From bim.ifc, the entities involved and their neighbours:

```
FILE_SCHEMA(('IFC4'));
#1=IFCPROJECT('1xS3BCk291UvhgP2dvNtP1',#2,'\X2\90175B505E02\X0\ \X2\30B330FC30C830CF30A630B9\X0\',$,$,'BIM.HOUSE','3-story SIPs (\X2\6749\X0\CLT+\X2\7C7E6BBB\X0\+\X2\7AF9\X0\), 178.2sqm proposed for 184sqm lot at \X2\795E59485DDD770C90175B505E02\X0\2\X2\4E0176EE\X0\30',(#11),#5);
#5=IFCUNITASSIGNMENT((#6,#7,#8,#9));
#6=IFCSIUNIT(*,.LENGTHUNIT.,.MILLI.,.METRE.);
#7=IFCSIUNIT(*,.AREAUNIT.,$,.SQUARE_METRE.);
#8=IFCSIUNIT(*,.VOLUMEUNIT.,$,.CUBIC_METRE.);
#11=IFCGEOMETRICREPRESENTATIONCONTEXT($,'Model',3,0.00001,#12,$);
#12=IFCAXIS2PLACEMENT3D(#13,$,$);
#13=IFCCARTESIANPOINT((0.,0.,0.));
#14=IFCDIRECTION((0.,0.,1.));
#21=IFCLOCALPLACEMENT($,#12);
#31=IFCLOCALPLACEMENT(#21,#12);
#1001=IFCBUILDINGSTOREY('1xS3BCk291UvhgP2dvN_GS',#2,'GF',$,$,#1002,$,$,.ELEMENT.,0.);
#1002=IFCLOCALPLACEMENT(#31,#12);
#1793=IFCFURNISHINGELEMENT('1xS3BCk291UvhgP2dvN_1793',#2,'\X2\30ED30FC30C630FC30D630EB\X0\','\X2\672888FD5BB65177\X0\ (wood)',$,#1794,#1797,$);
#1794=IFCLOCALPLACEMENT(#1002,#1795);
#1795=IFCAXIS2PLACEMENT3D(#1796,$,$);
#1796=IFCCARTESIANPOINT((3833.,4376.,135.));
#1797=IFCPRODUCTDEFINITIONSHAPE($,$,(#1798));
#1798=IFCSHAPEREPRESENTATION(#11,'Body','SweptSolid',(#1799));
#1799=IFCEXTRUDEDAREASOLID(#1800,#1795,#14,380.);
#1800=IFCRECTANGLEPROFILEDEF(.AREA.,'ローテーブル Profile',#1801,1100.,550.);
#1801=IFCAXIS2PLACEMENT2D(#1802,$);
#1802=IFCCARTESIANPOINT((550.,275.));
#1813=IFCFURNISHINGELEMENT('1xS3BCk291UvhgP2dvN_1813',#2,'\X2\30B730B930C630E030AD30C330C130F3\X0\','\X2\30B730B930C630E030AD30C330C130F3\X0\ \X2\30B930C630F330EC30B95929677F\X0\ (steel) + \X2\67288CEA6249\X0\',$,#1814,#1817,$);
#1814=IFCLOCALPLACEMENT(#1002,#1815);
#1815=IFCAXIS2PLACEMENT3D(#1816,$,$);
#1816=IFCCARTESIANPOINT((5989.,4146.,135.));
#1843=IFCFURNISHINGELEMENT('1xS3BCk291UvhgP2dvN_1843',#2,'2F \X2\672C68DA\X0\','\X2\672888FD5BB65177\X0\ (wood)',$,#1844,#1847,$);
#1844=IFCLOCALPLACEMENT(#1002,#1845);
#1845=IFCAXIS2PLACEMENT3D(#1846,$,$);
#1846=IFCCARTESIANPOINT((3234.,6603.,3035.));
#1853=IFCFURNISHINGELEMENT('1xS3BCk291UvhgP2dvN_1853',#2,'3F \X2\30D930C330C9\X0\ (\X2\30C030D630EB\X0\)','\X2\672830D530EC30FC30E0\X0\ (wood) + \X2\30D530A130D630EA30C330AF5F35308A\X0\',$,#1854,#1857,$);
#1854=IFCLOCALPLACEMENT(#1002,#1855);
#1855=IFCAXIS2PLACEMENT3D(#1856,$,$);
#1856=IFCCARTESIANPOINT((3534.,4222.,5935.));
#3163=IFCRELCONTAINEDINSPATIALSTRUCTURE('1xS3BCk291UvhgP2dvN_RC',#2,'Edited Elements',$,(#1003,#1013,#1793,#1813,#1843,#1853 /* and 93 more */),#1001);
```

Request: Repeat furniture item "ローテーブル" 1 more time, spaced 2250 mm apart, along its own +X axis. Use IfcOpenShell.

```python
import ifcopenshell
import ifcopenshell.api.geometry
import ifcopenshell.api.root
import ifcopenshell.util.element
import ifcopenshell.util.placement

model = ifcopenshell.open("bim.ifc")


def reuse_history(source, copy):
    """copy_class also copies each property set's owner history, people and application; keep the originals."""
    for rel in copy.IsDefinedBy:
        if rel.is_a("IfcRelDefinesByProperties") and (history := rel.RelatingPropertyDefinition.OwnerHistory):
            rel.RelatingPropertyDefinition.OwnerHistory = source.OwnerHistory
            ifcopenshell.util.element.remove_deep2(model, history)


source = model.by_id(1793)
base = ifcopenshell.util.placement.get_local_placement(source.ObjectPlacement)
step = base[:3, 0] * 2250.0

for i in range(1, 2):
    copy = ifcopenshell.api.root.copy_class(model, product=source)
    copy.Representation = ifcopenshell.util.element.copy_deep(
        model, source.Representation, exclude=["IfcGeometricRepresentationContext", "IfcRepresentationMap"]
    )
    reuse_history(source, copy)
    matrix = base.copy()
    matrix[:3, 3] += i * step
    print("added at", matrix[:3, 3].round(3) + 0.0)
    ifcopenshell.api.geometry.edit_object_placement(model, product=copy, matrix=matrix, is_si=False)

model.write("bim-out.ifc")
```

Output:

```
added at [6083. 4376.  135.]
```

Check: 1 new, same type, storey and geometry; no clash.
